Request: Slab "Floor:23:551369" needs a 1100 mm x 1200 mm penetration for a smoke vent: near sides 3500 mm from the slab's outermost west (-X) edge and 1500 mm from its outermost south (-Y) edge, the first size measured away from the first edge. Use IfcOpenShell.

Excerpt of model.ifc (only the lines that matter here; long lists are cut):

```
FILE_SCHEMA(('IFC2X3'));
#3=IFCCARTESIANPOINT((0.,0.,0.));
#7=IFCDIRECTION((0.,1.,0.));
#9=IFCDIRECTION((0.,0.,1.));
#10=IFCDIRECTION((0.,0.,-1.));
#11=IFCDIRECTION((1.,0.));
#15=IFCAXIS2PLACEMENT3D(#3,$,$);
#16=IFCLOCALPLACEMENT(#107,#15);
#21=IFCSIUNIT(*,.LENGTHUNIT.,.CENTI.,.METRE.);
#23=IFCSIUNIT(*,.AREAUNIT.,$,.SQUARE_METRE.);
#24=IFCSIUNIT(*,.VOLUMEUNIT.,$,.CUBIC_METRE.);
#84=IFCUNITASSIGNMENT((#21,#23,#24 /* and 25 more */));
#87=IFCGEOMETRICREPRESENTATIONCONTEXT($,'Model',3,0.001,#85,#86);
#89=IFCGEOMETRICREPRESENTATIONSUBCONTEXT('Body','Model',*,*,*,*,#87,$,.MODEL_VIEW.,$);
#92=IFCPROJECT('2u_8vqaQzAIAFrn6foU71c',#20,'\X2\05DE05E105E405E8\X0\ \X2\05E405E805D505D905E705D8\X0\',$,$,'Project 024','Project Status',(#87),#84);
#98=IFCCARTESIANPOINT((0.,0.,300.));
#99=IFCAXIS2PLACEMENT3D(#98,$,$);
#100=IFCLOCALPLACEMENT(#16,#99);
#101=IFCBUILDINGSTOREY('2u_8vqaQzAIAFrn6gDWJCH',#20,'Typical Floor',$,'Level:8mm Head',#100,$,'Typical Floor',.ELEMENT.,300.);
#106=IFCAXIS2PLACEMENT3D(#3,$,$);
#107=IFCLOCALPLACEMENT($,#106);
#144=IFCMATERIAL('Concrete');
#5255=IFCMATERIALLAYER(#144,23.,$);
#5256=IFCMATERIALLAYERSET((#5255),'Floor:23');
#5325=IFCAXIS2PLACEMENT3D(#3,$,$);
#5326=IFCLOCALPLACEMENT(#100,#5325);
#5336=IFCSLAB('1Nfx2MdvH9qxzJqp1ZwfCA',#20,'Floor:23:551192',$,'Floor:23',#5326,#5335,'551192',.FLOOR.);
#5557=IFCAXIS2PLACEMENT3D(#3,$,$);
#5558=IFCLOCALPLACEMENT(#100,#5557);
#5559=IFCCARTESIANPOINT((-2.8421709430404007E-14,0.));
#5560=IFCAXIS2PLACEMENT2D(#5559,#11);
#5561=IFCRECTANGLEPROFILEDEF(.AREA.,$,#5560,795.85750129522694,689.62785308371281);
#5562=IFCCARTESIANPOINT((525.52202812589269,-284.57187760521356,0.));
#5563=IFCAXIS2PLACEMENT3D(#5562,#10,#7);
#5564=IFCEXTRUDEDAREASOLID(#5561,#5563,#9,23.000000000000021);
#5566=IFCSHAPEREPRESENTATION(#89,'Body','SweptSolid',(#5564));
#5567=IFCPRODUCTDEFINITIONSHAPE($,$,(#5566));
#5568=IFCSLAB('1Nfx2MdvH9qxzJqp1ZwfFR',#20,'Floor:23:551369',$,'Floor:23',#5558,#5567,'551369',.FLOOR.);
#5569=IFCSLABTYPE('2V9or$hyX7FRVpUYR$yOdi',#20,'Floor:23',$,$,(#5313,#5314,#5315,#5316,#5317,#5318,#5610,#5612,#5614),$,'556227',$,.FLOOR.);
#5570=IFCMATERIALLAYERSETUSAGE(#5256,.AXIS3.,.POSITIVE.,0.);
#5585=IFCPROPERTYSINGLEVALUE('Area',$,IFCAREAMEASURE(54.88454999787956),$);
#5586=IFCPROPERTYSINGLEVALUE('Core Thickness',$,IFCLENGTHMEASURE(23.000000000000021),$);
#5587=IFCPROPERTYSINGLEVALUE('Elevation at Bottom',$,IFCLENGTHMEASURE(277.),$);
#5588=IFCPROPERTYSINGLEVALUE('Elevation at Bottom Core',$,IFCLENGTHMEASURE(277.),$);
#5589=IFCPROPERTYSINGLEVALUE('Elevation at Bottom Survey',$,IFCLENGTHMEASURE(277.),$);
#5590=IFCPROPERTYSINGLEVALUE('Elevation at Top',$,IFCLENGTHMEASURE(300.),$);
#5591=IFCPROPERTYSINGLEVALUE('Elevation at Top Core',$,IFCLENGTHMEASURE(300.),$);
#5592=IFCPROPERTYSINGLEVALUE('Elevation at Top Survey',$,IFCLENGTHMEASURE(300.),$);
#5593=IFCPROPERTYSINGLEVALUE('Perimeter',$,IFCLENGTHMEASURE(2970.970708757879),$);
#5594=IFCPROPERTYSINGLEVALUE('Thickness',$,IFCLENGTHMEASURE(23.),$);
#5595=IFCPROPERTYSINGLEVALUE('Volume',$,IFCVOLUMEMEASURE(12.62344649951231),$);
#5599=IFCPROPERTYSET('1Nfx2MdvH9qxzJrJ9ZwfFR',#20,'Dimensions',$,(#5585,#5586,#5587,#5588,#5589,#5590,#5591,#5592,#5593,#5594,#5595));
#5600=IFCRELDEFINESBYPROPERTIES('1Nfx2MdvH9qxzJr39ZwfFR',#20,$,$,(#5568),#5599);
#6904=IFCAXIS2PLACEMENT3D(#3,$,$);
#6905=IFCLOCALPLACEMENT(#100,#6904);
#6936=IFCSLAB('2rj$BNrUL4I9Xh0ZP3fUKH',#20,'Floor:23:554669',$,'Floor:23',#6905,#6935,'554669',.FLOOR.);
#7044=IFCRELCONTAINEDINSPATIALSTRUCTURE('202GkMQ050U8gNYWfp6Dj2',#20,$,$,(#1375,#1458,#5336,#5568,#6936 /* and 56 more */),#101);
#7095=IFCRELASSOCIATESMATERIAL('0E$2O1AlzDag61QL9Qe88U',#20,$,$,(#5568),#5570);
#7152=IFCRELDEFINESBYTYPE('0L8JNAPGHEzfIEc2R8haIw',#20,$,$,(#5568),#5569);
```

```python
import numpy as np
import ifcopenshell
import ifcopenshell.api.feature
import ifcopenshell.api.geometry
import ifcopenshell.api.pset
import ifcopenshell.api.root
import ifcopenshell.geom
import ifcopenshell.util.element
import ifcopenshell.util.placement
import ifcopenshell.util.representation
import ifcopenshell.util.shape
import ifcopenshell.util.unit

model = ifcopenshell.open("model.ifc")
unit_scale = ifcopenshell.util.unit.calculate_unit_scale(model)
area_scale = ifcopenshell.util.unit.calculate_unit_scale(model, "AREAUNIT")
volume_scale = ifcopenshell.util.unit.calculate_unit_scale(model, "VOLUMEUNIT")
settings = ifcopenshell.geom.settings()


def volume(element):
    """Net volume in cubic metres, openings subtracted."""
    shape = ifcopenshell.geom.create_shape(settings, element)
    return ifcopenshell.util.shape.get_volume(shape.geometry)


slab = model.by_guid("1Nfx2MdvH9qxzJqp1ZwfFR")
before = volume(slab)

# Extent in the slab's own axes, in metres. The edges named are its -X and -Y sides.
slab_shape = ifcopenshell.geom.create_shape(settings, slab)
vertices = ifcopenshell.util.shape.get_vertices(slab_shape.geometry)
x_min, y_min, bottom = vertices.min(axis=0)
top = vertices[:, 2].max()

opening = ifcopenshell.api.root.create_entity(model, ifc_class="IfcOpeningElement", name="Smoke vent opening")
context = ifcopenshell.util.representation.get_context(model, "Model", "Body", "MODEL_VIEW")
width, depth = 1.1, 1.2
outline = [(0.0, 0.0), (width, 0.0), (width, depth), (0.0, depth), (0.0, 0.0)]
# Overshoot both faces by 50 mm so the cut is clean.
shape = ifcopenshell.api.geometry.add_slab_representation(
    model, context=context, depth=top - bottom + 0.1, polyline=outline
)
ifcopenshell.api.geometry.assign_representation(model, product=opening, representation=shape)

matrix = ifcopenshell.util.placement.get_local_placement(slab.ObjectPlacement)
matrix[:, 3] = matrix @ np.append(np.array([x_min + 3.5, y_min + 1.5, bottom - 0.05]) / unit_scale, 1.0)
ifcopenshell.api.geometry.edit_object_placement(model, product=opening, matrix=matrix, is_si=False)
ifcopenshell.api.feature.add_feature(model, feature=opening, element=slab)

after = volume(slab)

# Update the slab's stored quantities.
pset = model.by_id(ifcopenshell.util.element.get_pset(slab, "Dimensions", should_inherit=False)["id"])
ifcopenshell.api.pset.edit_pset(model, pset=pset, properties={
    "Area": model.create_entity("IfcAreaMeasure", after / (top - bottom) / area_scale),
    "Volume": model.create_entity("IfcVolumeMeasure", after / volume_scale),
})

print(f"slab volume {before:.3f} -> {after:.3f} m3")

model.write("model_v2.ifc")
```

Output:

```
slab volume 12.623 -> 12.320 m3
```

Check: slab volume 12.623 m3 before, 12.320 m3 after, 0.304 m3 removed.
